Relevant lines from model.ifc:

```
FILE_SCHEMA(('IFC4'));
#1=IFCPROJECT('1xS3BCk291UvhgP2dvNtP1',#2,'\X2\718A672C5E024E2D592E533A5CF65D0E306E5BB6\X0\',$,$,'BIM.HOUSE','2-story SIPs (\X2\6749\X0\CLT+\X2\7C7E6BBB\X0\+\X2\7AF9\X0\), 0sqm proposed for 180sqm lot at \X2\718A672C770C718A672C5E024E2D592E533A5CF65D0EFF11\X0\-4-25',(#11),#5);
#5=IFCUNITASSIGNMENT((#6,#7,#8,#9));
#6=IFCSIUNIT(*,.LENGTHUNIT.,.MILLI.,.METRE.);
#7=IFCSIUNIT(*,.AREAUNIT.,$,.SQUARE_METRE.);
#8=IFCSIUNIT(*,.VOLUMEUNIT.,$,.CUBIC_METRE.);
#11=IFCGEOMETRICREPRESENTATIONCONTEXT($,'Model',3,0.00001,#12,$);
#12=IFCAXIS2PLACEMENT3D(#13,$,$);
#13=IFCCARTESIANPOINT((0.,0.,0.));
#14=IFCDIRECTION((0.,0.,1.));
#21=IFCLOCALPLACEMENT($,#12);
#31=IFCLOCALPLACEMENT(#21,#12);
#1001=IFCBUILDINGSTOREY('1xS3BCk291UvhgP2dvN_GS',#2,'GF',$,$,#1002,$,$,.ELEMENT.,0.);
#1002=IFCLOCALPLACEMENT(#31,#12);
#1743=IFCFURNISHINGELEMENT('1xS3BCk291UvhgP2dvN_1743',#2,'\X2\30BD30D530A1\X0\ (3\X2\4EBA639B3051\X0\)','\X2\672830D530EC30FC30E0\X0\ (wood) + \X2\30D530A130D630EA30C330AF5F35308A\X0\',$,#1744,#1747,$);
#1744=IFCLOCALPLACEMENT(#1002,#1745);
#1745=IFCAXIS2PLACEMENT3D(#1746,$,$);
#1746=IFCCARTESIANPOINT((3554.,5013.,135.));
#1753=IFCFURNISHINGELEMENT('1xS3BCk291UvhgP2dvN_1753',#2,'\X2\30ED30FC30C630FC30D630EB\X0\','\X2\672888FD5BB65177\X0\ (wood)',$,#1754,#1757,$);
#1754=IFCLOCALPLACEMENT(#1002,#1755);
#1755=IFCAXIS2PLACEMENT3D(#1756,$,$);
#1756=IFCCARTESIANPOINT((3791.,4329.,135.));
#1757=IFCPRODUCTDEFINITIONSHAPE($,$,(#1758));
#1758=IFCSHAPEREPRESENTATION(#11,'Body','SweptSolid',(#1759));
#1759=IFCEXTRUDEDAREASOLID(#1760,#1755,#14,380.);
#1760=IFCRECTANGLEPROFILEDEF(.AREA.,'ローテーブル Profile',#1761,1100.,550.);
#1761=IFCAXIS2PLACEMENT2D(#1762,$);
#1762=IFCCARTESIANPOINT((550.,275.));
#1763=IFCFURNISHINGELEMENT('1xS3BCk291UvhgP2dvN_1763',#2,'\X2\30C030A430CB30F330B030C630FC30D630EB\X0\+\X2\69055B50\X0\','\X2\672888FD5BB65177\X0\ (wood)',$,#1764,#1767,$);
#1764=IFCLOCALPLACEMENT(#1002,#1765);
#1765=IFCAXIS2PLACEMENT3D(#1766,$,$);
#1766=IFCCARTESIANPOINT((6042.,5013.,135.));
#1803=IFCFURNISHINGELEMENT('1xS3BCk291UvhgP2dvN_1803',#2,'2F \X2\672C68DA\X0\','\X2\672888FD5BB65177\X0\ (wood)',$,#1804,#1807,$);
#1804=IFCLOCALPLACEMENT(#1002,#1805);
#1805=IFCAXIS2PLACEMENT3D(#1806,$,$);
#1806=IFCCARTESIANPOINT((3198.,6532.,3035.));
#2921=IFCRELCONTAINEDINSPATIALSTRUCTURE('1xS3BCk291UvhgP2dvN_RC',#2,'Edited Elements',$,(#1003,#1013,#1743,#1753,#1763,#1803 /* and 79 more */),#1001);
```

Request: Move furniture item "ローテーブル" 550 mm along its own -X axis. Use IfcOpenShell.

```python
import ifcopenshell
import ifcopenshell.api.geometry
import ifcopenshell.util.placement
import ifcopenshell.util.unit

model = ifcopenshell.open("model.ifc")
unit_scale = ifcopenshell.util.unit.calculate_unit_scale(model)

item = model.by_id(1753)
matrix = ifcopenshell.util.placement.get_local_placement(item.ObjectPlacement)
matrix[:3, 3] -= matrix[:3, 0] * 0.55 / unit_scale
ifcopenshell.api.geometry.edit_object_placement(model, product=item, matrix=matrix, is_si=False)

print(ifcopenshell.util.placement.get_local_placement(item.ObjectPlacement).round(3) + 0.0)

model.write("model_edited.ifc")
```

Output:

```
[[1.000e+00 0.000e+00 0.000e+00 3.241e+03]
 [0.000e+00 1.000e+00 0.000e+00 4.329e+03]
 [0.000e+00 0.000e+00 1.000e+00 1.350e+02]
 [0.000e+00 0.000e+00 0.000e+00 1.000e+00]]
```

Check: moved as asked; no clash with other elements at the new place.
